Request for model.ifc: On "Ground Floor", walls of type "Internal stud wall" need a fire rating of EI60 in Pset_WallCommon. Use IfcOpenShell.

First a look at what the model holds.

```python
import ifcopenshell
import ifcopenshell.util.element

model = ifcopenshell.open("model.ifc")
print(model.schema)
storey = next(s for s in model.by_type("IfcBuildingStorey") if s.Name == "Ground Floor")
walls = [e for e in ifcopenshell.util.element.get_decomposition(storey) if e.is_a("IfcWall")]
seen = {}
for e in walls:
    element_type = ifcopenshell.util.element.get_type(e)
    key = (element_type.Name if element_type != e and element_type else None, ifcopenshell.util.element.get_pset(e, "Pset_WallCommon", "FireRating"))
    seen[key] = seen.get(key, 0) + 1
for (name, value), count in sorted(seen.items(), key=str):
    print(count, "x", name, "|", value)
```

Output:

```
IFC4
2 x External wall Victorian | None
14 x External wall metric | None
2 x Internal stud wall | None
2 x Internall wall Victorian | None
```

```python
import ifcopenshell
import ifcopenshell.api.pset
import ifcopenshell.util.element

model = ifcopenshell.open("model.ifc")

storey = next(s for s in model.by_type("IfcBuildingStorey") if s.Name == "Ground Floor")
walls = [e for e in ifcopenshell.util.element.get_decomposition(storey) if e.is_a("IfcWall")]

count = 0
for e in walls:
    element_type = ifcopenshell.util.element.get_type(e)
    if element_type in (None, e) or element_type.Name != "Internal stud wall":
        continue
    # add_pset returns the element's existing set when there is one.
    pset = ifcopenshell.api.pset.add_pset(model, product=e, name="Pset_WallCommon")
    ifcopenshell.api.pset.edit_pset(model, pset=pset, properties={"FireRating": "EI60"})
    count += 1

print(count, "walls updated")

model.write("model_updated.ifc")
```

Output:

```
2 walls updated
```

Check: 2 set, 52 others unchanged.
